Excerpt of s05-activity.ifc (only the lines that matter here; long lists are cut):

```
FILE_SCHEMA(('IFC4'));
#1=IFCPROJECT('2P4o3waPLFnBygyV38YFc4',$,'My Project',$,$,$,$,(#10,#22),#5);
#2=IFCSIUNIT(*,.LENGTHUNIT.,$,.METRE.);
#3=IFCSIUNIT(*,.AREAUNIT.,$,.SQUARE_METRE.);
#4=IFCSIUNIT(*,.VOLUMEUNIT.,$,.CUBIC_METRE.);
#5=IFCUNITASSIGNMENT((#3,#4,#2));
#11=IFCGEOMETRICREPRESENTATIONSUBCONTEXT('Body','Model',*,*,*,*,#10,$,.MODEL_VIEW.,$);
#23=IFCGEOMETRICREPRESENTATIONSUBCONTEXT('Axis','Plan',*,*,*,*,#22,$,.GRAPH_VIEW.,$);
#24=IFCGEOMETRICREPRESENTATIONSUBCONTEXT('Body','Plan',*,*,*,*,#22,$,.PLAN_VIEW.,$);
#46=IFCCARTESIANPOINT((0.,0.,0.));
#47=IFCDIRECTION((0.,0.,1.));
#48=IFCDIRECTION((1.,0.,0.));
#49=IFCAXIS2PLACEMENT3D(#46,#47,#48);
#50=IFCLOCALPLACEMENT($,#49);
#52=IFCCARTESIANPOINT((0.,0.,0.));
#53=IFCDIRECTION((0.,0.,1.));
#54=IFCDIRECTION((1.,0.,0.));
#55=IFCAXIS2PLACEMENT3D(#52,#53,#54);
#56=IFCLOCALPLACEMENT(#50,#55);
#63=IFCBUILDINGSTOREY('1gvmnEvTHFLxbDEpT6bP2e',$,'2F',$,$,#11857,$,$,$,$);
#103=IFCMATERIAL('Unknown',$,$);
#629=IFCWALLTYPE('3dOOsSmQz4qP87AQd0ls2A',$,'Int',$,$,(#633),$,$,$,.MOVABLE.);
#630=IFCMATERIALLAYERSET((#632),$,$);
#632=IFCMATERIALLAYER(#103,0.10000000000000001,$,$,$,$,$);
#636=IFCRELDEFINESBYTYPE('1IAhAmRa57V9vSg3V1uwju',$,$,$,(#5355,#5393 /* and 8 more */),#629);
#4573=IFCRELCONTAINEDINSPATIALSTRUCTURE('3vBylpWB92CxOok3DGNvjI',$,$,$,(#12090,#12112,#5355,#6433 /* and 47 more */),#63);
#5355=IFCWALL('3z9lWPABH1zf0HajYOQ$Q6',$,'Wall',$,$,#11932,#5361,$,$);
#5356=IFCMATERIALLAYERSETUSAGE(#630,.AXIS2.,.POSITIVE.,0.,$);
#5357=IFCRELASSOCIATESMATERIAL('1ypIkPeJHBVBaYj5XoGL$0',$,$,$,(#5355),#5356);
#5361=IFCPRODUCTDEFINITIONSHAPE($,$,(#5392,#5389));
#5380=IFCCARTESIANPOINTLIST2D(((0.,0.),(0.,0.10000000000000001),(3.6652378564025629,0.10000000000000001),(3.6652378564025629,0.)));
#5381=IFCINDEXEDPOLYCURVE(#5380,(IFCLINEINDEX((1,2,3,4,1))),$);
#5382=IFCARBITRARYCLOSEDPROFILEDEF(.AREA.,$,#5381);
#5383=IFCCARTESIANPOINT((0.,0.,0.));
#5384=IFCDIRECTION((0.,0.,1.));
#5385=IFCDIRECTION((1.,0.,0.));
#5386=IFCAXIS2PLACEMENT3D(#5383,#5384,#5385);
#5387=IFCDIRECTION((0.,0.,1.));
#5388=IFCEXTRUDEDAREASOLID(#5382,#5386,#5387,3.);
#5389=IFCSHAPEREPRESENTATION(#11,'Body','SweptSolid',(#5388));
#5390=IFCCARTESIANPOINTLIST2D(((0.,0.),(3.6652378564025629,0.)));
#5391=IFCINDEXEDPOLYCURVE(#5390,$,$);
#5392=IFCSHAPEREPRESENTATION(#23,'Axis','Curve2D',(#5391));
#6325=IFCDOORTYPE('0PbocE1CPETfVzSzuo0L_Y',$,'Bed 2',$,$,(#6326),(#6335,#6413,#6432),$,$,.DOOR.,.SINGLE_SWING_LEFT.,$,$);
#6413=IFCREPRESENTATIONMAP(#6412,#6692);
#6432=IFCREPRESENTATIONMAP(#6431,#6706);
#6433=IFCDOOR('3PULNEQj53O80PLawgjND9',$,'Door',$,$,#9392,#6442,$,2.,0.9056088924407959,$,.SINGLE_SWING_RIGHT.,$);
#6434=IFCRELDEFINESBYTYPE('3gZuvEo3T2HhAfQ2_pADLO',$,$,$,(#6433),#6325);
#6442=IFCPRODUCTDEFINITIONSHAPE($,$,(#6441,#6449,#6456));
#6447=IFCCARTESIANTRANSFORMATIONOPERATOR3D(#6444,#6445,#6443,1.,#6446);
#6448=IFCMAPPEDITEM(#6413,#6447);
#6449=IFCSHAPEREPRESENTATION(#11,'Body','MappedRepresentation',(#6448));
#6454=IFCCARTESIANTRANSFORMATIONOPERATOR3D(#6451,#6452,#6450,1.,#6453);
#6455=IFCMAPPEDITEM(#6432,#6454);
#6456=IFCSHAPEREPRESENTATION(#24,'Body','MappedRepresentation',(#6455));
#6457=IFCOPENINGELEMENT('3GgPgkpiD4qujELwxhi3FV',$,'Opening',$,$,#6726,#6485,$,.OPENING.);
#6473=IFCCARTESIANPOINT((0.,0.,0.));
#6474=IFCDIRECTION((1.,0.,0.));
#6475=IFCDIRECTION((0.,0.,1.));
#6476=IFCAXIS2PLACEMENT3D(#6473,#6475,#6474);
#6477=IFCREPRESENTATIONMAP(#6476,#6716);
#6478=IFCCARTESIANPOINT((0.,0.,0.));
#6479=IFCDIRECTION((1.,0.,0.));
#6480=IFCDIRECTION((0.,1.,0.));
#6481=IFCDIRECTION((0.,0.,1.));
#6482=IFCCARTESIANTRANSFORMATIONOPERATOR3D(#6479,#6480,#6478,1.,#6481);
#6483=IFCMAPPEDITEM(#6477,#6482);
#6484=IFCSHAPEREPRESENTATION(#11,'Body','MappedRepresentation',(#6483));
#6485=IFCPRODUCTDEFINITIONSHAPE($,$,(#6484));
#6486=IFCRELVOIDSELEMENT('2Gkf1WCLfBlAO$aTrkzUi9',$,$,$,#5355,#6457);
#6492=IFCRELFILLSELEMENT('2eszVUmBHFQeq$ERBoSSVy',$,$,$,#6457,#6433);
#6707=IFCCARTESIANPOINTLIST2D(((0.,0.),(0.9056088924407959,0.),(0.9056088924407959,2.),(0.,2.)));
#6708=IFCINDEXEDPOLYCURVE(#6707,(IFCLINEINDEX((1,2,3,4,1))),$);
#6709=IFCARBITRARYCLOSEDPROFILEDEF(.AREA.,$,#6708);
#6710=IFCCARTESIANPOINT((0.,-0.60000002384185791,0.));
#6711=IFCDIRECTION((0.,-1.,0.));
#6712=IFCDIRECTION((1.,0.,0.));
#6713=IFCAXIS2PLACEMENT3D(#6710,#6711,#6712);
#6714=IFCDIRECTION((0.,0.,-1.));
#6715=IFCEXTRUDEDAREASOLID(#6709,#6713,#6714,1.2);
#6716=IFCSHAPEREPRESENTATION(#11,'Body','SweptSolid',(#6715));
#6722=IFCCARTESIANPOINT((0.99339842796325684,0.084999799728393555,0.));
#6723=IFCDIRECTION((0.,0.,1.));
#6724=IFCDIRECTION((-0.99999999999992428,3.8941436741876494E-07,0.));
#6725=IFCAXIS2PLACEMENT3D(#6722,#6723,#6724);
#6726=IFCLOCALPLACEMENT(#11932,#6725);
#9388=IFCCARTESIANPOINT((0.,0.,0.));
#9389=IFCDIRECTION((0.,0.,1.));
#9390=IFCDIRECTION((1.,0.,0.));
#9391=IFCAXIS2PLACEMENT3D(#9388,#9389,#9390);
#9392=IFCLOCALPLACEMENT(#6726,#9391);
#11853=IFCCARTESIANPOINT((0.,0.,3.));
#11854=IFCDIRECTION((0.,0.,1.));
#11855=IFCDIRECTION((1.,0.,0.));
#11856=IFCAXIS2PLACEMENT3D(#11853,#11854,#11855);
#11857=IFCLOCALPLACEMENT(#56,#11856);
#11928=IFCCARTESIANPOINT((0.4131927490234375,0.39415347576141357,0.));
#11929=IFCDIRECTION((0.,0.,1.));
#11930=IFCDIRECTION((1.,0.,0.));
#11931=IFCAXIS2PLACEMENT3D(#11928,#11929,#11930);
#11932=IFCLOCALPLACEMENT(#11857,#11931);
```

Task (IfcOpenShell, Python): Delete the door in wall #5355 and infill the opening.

```python
import ifcopenshell
import ifcopenshell.api.feature
import ifcopenshell.api.root
import ifcopenshell.geom
import ifcopenshell.util.shape

model = ifcopenshell.open("s05-activity.ifc")
settings = ifcopenshell.geom.settings()


def volume(element):
    """Net volume in cubic metres, openings subtracted."""
    shape = ifcopenshell.geom.create_shape(settings, element)
    return ifcopenshell.util.shape.get_volume(shape.geometry)


door = model.by_guid("3PULNEQj53O80PLawgjND9")
opening = door.FillsVoids[0].RelatingOpeningElement
wall = opening.VoidsElements[0].RelatingBuildingElement
before = volume(wall)

ifcopenshell.api.root.remove_product(model, product=door)
ifcopenshell.api.feature.remove_feature(model, feature=opening)

after = volume(wall)

print(f"wall volume {before:.3f} -> {after:.3f} m3")

model.write("s05-activity_v2.ifc")
```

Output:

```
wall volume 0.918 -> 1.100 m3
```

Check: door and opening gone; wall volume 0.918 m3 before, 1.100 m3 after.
